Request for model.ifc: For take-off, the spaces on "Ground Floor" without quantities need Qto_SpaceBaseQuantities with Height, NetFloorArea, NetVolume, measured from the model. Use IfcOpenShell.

First a look at what the model holds.

```python
import ifcopenshell
import ifcopenshell.util.element
import ifcopenshell.util.unit

model = ifcopenshell.open("model.ifc")
print(model.schema)
for unit_type in ("LENGTHUNIT", "AREAUNIT", "VOLUMEUNIT"):
    print(unit_type, ifcopenshell.util.unit.calculate_unit_scale(model, unit_type))
storey = next(s for s in model.by_type("IfcBuildingStorey") if s.Name == "Ground Floor")
spaces = [e for e in ifcopenshell.util.element.get_decomposition(storey) if e.is_a("IfcSpace")]
for e in sorted(spaces, key=lambda e: e.id()):
    print(e.id(), e.is_a(), e.Name, list(ifcopenshell.util.element.get_psets(e, qtos_only=True)), sep=" | ")
```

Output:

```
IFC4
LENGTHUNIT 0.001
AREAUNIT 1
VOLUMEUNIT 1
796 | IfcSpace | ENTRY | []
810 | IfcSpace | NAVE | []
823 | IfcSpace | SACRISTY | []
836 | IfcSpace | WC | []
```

```python
import ifcopenshell
import ifcopenshell.api.pset
import ifcopenshell.geom
import ifcopenshell.util.element
import ifcopenshell.util.shape
import ifcopenshell.util.unit

model = ifcopenshell.open("model.ifc")
unit_scale = ifcopenshell.util.unit.calculate_unit_scale(model)
area_scale = ifcopenshell.util.unit.calculate_unit_scale(model, "AREAUNIT")
volume_scale = ifcopenshell.util.unit.calculate_unit_scale(model, "VOLUMEUNIT")
settings = ifcopenshell.geom.settings()

storey = next(s for s in model.by_type("IfcBuildingStorey") if s.Name == "Ground Floor")
spaces = [e for e in ifcopenshell.util.element.get_decomposition(storey) if e.is_a("IfcSpace")]

for e in sorted(spaces, key=lambda e: e.id()):
    if ifcopenshell.util.element.get_psets(e, qtos_only=True, should_inherit=False):
        continue
    # Geometry comes back in metres, in the element's own axes.
    shape = ifcopenshell.geom.create_shape(settings, e)
    values = {
        "Height": ifcopenshell.util.shape.get_z(shape.geometry) / unit_scale,
        "NetFloorArea": ifcopenshell.util.shape.get_footprint_area(shape.geometry) / area_scale,
        "NetVolume": ifcopenshell.util.shape.get_volume(shape.geometry) / volume_scale,
    }
    qto = ifcopenshell.api.pset.add_qto(model, product=e, name="Qto_SpaceBaseQuantities")
    ifcopenshell.api.pset.edit_qto(model, qto=qto, properties=values)
    print(e.id(), {k: round(v, 3) for k, v in values.items()})

model.write("model_rev.ifc")
```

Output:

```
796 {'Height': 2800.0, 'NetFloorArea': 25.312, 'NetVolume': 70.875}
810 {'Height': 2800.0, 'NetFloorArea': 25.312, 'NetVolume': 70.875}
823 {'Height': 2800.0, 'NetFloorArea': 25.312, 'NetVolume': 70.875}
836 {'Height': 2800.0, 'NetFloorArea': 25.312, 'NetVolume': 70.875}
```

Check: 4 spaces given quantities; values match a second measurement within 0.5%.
